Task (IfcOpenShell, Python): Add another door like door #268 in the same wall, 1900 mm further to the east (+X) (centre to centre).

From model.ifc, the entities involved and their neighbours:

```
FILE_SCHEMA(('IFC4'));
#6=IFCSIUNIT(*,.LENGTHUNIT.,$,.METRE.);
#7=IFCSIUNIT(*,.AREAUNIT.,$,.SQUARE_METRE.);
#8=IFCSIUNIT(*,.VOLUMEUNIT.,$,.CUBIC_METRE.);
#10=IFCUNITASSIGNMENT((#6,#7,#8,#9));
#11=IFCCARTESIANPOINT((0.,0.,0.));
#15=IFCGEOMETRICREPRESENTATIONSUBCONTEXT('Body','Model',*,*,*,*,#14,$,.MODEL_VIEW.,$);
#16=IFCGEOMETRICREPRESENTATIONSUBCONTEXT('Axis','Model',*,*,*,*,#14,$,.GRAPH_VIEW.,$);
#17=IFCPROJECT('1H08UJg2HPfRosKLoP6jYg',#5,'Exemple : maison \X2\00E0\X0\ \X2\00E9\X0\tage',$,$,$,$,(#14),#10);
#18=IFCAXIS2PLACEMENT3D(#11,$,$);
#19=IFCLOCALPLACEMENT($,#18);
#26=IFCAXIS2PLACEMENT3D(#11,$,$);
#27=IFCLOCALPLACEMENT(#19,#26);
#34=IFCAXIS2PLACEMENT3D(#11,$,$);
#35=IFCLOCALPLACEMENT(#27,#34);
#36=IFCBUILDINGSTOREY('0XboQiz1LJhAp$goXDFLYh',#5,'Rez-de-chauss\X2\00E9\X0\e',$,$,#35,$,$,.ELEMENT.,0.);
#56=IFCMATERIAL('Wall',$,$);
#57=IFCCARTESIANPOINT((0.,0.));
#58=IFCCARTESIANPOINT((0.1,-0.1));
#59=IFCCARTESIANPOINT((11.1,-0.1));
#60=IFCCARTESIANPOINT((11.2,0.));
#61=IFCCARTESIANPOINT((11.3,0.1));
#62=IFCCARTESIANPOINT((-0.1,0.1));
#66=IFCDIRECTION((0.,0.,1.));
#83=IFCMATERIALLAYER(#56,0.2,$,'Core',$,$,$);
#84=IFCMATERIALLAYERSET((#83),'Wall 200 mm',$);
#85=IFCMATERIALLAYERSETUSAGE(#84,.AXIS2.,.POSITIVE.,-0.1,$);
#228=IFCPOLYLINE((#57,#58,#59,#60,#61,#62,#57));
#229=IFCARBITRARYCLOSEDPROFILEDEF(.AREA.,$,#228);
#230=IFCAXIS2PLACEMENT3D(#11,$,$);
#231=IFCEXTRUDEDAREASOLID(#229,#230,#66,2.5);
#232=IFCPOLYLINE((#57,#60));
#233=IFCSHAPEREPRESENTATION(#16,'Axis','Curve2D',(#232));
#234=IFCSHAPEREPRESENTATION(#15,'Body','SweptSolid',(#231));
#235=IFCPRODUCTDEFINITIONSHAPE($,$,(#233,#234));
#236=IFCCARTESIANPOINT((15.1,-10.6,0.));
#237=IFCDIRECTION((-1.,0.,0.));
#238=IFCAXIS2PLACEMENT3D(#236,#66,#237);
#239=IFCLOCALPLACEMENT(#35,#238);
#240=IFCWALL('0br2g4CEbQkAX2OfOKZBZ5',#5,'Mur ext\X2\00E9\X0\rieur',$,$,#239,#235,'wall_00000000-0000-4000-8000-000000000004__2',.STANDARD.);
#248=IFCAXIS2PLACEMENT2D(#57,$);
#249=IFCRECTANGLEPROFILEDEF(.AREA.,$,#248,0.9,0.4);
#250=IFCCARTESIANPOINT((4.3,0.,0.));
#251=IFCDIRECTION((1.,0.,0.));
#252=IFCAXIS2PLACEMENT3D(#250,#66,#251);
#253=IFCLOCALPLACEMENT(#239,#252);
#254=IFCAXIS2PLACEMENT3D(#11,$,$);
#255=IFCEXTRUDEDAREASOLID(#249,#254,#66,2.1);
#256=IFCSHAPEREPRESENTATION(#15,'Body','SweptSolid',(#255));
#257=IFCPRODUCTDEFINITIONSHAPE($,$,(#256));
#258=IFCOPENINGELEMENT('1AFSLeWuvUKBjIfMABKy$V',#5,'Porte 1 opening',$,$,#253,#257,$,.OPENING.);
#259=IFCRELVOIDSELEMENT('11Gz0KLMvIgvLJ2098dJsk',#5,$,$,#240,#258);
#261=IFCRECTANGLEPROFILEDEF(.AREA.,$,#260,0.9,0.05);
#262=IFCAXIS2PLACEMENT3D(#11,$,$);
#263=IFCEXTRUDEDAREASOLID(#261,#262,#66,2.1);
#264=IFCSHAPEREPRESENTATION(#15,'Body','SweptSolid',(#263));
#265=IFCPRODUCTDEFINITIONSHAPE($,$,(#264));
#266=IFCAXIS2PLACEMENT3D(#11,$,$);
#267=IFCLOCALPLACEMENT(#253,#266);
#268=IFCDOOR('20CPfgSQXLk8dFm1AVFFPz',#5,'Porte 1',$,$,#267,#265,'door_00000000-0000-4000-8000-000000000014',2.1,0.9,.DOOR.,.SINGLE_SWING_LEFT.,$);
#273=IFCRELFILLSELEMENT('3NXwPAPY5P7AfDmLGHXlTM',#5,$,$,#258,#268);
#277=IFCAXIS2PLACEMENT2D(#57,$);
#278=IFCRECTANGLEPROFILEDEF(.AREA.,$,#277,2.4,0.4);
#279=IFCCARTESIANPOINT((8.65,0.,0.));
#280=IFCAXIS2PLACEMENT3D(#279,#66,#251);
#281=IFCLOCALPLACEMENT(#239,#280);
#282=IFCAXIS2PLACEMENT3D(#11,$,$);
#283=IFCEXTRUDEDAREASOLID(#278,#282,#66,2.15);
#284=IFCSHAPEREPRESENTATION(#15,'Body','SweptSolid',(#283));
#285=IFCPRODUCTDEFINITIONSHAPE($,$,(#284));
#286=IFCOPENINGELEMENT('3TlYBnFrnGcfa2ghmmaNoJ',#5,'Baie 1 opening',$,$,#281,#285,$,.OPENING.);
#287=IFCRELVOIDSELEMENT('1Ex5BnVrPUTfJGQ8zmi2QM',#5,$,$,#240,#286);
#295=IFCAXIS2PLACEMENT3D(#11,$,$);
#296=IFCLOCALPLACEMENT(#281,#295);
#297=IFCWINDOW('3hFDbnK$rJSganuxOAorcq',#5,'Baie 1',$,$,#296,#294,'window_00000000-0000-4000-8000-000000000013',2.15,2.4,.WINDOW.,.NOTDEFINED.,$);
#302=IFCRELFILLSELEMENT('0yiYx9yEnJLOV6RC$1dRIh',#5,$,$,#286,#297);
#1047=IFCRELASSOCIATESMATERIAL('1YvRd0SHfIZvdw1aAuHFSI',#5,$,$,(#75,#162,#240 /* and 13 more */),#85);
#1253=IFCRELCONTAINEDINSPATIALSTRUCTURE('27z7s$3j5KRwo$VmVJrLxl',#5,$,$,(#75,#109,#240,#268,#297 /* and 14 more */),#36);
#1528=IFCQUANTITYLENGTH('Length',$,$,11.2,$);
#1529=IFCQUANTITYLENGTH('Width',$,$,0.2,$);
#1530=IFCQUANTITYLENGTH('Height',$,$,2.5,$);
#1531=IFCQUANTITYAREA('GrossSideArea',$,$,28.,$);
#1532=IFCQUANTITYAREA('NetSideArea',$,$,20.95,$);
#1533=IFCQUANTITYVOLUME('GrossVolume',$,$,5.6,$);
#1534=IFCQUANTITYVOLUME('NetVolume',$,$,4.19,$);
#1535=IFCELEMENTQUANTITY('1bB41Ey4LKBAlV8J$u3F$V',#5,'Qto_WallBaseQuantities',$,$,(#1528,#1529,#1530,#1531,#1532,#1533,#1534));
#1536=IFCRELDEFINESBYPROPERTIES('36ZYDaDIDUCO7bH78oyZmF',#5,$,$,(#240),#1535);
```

```python
import ifcopenshell
import ifcopenshell.api.feature
import ifcopenshell.api.geometry
import ifcopenshell.api.pset
import ifcopenshell.api.root
import ifcopenshell.geom
import ifcopenshell.util.element
import ifcopenshell.util.placement
import ifcopenshell.util.shape
import ifcopenshell.util.unit

model = ifcopenshell.open("model.ifc")
unit_scale = ifcopenshell.util.unit.calculate_unit_scale(model)
area_scale = ifcopenshell.util.unit.calculate_unit_scale(model, "AREAUNIT")
volume_scale = ifcopenshell.util.unit.calculate_unit_scale(model, "VOLUMEUNIT")
settings = ifcopenshell.geom.settings()


def volume(element):
    """Net volume in cubic metres, openings subtracted."""
    shape = ifcopenshell.geom.create_shape(settings, element)
    return ifcopenshell.util.shape.get_volume(shape.geometry)


def reuse_history(source, copy):
    """copy_class also copies each property set's owner history, people and application; keep the originals."""
    for rel in copy.IsDefinedBy:
        if rel.is_a("IfcRelDefinesByProperties") and (history := rel.RelatingPropertyDefinition.OwnerHistory):
            rel.RelatingPropertyDefinition.OwnerHistory = source.OwnerHistory
            ifcopenshell.util.element.remove_deep2(model, history)


door = model.by_guid("20CPfgSQXLk8dFm1AVFFPz")
opening = door.FillsVoids[0].RelatingOpeningElement
wall = opening.VoidsElements[0].RelatingBuildingElement
before = volume(wall)
shift = ifcopenshell.util.placement.get_local_placement(wall.ObjectPlacement)[:3, 0] * -1.9 / unit_scale

# copy_class copies the void relationship, type, container and properties, but no geometry.
new_opening = ifcopenshell.api.root.copy_class(model, product=opening)
new_opening.Representation = ifcopenshell.util.element.copy_deep(
    model, opening.Representation, exclude=["IfcGeometricRepresentationContext", "IfcRepresentationMap"]
)
new_door = ifcopenshell.api.root.copy_class(model, product=door)
new_door.Representation = ifcopenshell.util.element.copy_deep(
    model, door.Representation, exclude=["IfcGeometricRepresentationContext", "IfcRepresentationMap"]
)
new_door.Tag = None
reuse_history(door, new_door)
ifcopenshell.api.feature.add_filling(model, opening=new_opening, element=new_door)

for old, new in ((opening, new_opening), (door, new_door)):
    matrix = ifcopenshell.util.placement.get_local_placement(old.ObjectPlacement)
    matrix[:3, 3] += shift
    ifcopenshell.api.geometry.edit_object_placement(model, product=new, matrix=matrix, is_si=False)

after = volume(wall)
thickness = 0.2  # wall thickness in metres

# Update the wall's stored quantities.
qto = model.by_id(ifcopenshell.util.element.get_pset(wall, "Qto_WallBaseQuantities", should_inherit=False)["id"])
ifcopenshell.api.pset.edit_qto(model, qto=qto, properties={
    "NetSideArea": after / thickness / area_scale,
    "NetVolume": after / volume_scale,
})

print(f"wall volume {before:.3f} -> {after:.3f} m3")

model.write("model_rev.ifc")
```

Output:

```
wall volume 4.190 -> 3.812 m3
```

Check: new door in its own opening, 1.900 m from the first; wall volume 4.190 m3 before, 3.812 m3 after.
